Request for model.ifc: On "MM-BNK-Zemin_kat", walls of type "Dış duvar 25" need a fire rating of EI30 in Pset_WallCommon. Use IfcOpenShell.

First a look at what the model holds.

```python
import ifcopenshell
import ifcopenshell.util.element

model = ifcopenshell.open("model.ifc")
print(model.schema)
storey = next(s for s in model.by_type("IfcBuildingStorey") if s.Name == "MM-BNK-Zemin_kat")
walls = [e for e in ifcopenshell.util.element.get_decomposition(storey) if e.is_a("IfcWall")]
seen = {}
for e in walls:
    element_type = ifcopenshell.util.element.get_type(e)
    key = (element_type.Name if element_type != e and element_type else None, ifcopenshell.util.element.get_pset(e, "Pset_WallCommon", "FireRating"))
    seen[key] = seen.get(key, 0) + 1
for (name, value), count in sorted(seen.items(), key=str):
    print(count, "x", name, "|", value)
```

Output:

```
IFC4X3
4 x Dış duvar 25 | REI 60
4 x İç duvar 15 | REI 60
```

```python
import ifcopenshell
import ifcopenshell.api.pset
import ifcopenshell.util.element

model = ifcopenshell.open("model.ifc")

storey = next(s for s in model.by_type("IfcBuildingStorey") if s.Name == "MM-BNK-Zemin_kat")
walls = [e for e in ifcopenshell.util.element.get_decomposition(storey) if e.is_a("IfcWall")]

count = 0
for e in walls:
    element_type = ifcopenshell.util.element.get_type(e)
    if element_type in (None, e) or element_type.Name != "Dış duvar 25":
        continue
    # add_pset returns the element's existing set when there is one.
    pset = ifcopenshell.api.pset.add_pset(model, product=e, name="Pset_WallCommon")
    ifcopenshell.api.pset.edit_pset(model, pset=pset, properties={"FireRating": "EI30"})
    count += 1

print(count, "walls updated")

model.write("model-out.ifc")
```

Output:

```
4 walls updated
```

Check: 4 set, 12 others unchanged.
